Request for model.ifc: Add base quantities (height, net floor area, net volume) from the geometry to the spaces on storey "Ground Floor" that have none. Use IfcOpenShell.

First a look at what the model holds.

```python
import ifcopenshell
import ifcopenshell.util.element
import ifcopenshell.util.unit

model = ifcopenshell.open("model.ifc")
print(model.schema)
for unit_type in ("LENGTHUNIT", "AREAUNIT", "VOLUMEUNIT"):
    print(unit_type, ifcopenshell.util.unit.calculate_unit_scale(model, unit_type))
storey = next(s for s in model.by_type("IfcBuildingStorey") if s.Name == "Ground Floor")
spaces = [e for e in ifcopenshell.util.element.get_decomposition(storey) if e.is_a("IfcSpace")]
for e in sorted(spaces, key=lambda e: e.id()):
    print(e.id(), e.is_a(), e.Name, list(ifcopenshell.util.element.get_psets(e, qtos_only=True)), sep=" | ")
```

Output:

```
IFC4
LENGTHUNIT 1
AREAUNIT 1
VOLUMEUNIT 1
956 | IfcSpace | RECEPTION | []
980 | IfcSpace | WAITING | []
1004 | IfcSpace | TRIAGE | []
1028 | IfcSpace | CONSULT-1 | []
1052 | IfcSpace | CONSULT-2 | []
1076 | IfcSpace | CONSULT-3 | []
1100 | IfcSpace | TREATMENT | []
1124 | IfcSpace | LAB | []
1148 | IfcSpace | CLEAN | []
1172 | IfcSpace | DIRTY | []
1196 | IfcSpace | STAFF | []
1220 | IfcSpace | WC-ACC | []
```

```python
import ifcopenshell
import ifcopenshell.api.pset
import ifcopenshell.geom
import ifcopenshell.util.element
import ifcopenshell.util.shape
import ifcopenshell.util.unit

model = ifcopenshell.open("model.ifc")
unit_scale = ifcopenshell.util.unit.calculate_unit_scale(model)
area_scale = ifcopenshell.util.unit.calculate_unit_scale(model, "AREAUNIT")
volume_scale = ifcopenshell.util.unit.calculate_unit_scale(model, "VOLUMEUNIT")
settings = ifcopenshell.geom.settings()

storey = next(s for s in model.by_type("IfcBuildingStorey") if s.Name == "Ground Floor")
spaces = [e for e in ifcopenshell.util.element.get_decomposition(storey) if e.is_a("IfcSpace")]

for e in sorted(spaces, key=lambda e: e.id()):
    if ifcopenshell.util.element.get_psets(e, qtos_only=True, should_inherit=False):
        continue
    # Geometry comes back in metres, in the element's own axes.
    shape = ifcopenshell.geom.create_shape(settings, e)
    values = {
        "Height": ifcopenshell.util.shape.get_z(shape.geometry) / unit_scale,
        "NetFloorArea": ifcopenshell.util.shape.get_footprint_area(shape.geometry) / area_scale,
        "NetVolume": ifcopenshell.util.shape.get_volume(shape.geometry) / volume_scale,
    }
    qto = ifcopenshell.api.pset.add_qto(model, product=e, name="Qto_SpaceBaseQuantities")
    ifcopenshell.api.pset.edit_qto(model, qto=qto, properties=values)
    print(e.id(), {k: round(v, 3) for k, v in values.items()})

model.write("model_rev.ifc")
```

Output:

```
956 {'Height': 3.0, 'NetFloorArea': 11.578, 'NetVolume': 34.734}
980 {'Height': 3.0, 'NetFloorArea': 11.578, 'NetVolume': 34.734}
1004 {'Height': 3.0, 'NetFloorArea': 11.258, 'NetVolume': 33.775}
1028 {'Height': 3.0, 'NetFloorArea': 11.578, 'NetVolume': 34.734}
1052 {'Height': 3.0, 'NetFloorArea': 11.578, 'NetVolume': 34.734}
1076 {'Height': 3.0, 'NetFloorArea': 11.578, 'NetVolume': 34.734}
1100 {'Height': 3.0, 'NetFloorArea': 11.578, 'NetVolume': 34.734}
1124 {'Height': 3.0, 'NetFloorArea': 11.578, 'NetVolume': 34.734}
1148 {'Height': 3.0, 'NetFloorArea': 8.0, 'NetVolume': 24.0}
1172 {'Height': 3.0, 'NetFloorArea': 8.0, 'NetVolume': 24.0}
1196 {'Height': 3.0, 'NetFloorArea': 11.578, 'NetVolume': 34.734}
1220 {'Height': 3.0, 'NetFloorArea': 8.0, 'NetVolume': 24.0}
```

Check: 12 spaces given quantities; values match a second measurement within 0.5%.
